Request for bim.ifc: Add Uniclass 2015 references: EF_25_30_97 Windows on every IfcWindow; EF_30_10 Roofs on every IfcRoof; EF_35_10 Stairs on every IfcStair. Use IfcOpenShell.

First a look at what the model holds.

```python
import ifcopenshell

model = ifcopenshell.open("bim.ifc")
print(model.schema)
print("classifications:", [c.Name for c in model.by_type("IfcClassification")])
for ifc_class in ("IfcDoor", "IfcRoof", "IfcStair", "IfcWall", "IfcWindow"):
    print(ifc_class, len(model.by_type(ifc_class)))
```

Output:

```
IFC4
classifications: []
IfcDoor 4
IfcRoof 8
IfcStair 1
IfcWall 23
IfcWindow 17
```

```python
import ifcopenshell
import ifcopenshell.api.classification

model = ifcopenshell.open("bim.ifc")

system = ifcopenshell.api.classification.add_classification(model, classification="Uniclass 2015")

codes = {
    "IfcWindow": ("EF_25_30_97", "Windows"),
    "IfcRoof": ("EF_30_10", "Roofs"),
    "IfcStair": ("EF_35_10", "Stairs"),
}
for ifc_class, (code, name) in codes.items():
    products = model.by_type(ifc_class)
    ifcopenshell.api.classification.add_reference(
        model, products=products, classification=system, identification=code, name=name
    )
    print(code, len(products))

model.write("bim-out.ifc")
```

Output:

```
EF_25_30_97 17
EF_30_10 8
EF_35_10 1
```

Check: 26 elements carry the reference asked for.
